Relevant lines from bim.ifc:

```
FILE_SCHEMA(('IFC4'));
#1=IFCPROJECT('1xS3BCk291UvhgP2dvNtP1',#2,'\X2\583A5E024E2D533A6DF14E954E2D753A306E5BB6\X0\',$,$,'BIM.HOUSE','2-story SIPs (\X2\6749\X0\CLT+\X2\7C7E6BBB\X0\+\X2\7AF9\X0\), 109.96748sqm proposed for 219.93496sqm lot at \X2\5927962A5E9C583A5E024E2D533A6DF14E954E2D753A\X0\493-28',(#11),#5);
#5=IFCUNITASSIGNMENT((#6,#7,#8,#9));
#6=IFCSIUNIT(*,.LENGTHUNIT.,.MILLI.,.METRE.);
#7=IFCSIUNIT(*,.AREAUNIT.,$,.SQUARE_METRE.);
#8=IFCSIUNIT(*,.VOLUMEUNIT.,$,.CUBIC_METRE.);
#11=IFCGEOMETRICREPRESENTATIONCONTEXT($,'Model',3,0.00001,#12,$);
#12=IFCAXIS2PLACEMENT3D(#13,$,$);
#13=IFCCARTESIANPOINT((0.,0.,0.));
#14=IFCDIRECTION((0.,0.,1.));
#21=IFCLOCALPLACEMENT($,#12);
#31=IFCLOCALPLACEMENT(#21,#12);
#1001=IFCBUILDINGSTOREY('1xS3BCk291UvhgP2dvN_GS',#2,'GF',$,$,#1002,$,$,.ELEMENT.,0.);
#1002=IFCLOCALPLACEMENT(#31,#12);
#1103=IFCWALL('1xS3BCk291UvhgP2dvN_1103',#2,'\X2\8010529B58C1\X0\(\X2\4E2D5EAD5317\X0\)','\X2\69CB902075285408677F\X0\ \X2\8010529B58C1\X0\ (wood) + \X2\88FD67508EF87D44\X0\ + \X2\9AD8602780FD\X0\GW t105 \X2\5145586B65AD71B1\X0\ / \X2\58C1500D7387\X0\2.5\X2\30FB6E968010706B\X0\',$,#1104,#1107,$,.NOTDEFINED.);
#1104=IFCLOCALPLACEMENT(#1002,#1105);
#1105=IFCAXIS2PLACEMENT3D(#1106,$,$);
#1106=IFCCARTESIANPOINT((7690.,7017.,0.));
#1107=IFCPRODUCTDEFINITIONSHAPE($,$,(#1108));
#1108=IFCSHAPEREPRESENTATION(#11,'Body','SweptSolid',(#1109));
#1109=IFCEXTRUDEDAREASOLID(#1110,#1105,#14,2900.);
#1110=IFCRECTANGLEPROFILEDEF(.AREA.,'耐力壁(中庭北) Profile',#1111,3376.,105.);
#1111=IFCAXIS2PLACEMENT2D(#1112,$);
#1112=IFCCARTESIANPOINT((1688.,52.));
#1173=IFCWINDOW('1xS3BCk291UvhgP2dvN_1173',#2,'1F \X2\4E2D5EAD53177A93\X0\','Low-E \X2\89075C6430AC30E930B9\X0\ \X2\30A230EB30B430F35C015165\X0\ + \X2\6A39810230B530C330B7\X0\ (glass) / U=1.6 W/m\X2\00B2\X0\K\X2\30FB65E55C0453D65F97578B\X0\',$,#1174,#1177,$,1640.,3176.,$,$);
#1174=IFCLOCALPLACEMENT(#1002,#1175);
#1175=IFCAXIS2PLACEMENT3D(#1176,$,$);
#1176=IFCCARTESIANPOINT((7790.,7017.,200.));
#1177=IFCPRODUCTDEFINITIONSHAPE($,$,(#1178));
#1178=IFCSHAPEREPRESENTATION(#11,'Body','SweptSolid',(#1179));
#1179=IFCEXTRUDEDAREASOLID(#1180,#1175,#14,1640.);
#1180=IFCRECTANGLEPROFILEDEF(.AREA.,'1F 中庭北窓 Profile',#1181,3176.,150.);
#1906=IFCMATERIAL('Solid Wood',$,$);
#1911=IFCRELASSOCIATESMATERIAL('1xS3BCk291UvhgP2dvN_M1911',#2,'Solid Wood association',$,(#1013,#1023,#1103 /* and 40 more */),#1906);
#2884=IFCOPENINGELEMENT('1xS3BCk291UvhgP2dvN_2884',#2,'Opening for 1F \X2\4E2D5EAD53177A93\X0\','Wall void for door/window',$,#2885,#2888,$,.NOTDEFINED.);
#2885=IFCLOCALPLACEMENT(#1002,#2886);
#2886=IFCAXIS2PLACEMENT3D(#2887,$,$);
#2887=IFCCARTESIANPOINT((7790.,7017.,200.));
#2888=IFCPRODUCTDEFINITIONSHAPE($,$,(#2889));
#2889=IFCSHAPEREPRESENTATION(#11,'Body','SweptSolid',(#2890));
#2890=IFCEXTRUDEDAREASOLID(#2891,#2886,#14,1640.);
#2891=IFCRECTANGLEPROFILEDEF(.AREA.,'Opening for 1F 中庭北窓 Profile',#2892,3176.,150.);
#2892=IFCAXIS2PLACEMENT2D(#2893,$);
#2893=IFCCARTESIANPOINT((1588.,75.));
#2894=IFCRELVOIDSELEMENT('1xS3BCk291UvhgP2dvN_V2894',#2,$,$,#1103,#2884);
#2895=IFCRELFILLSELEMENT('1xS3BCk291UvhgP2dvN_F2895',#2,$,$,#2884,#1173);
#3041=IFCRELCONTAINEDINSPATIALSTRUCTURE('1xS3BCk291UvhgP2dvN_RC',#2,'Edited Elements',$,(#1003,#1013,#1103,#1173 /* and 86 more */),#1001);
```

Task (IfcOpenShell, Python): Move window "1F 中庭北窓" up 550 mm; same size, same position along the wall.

```python
import numpy as np
import ifcopenshell
import ifcopenshell.api.geometry
import ifcopenshell.util.placement
import ifcopenshell.util.unit

model = ifcopenshell.open("bim.ifc")
unit_scale = ifcopenshell.util.unit.calculate_unit_scale(model)

window = model.by_guid("1xS3BCk291UvhgP2dvN_1173")
opening = window.FillsVoids[0].RelatingOpeningElement
dz = 550.0

shift = np.array([0.0, 0.0, dz])
# The window is not placed relative to its opening, so move both.
for product in (opening, window):
    matrix = ifcopenshell.util.placement.get_local_placement(product.ObjectPlacement)
    matrix[:3, 3] += shift
    ifcopenshell.api.geometry.edit_object_placement(model, product=product, matrix=matrix, is_si=False)

print(f"moved by {dz * unit_scale:+.3f} m")

model.write("bim_rev.ifc")
```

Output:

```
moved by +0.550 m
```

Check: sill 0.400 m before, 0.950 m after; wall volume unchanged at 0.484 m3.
